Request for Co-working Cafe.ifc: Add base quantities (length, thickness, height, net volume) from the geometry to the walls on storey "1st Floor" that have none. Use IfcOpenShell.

First a look at what the model holds.

```python
import ifcopenshell
import ifcopenshell.util.element
import ifcopenshell.util.unit

model = ifcopenshell.open("Co-working Cafe.ifc")
print(model.schema)
for unit_type in ("LENGTHUNIT", "AREAUNIT", "VOLUMEUNIT"):
    print(unit_type, ifcopenshell.util.unit.calculate_unit_scale(model, unit_type))
storey = next(s for s in model.by_type("IfcBuildingStorey") if s.Name == "1st Floor")
walls = [e for e in ifcopenshell.util.element.get_decomposition(storey) if e.is_a("IfcWall")]
for e in sorted(walls, key=lambda e: e.id()):
    print(e.id(), e.is_a(), e.Name, list(ifcopenshell.util.element.get_psets(e, qtos_only=True)), sep=" | ")
```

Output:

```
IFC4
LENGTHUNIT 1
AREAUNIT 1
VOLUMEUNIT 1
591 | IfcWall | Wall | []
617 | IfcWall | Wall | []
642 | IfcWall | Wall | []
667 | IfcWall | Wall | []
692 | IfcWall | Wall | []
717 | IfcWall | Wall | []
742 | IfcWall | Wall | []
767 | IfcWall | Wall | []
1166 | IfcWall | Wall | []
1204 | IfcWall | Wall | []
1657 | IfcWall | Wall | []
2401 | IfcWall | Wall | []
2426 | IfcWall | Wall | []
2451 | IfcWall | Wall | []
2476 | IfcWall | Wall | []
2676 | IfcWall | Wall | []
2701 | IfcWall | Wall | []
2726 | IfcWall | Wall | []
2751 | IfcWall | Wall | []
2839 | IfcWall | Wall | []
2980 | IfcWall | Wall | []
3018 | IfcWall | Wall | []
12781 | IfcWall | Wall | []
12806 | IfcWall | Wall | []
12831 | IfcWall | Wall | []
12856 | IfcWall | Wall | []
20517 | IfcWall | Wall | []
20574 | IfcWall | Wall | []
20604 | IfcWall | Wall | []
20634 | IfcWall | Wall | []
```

```python
import ifcopenshell
import ifcopenshell.api.pset
import ifcopenshell.geom
import ifcopenshell.util.element
import ifcopenshell.util.shape
import ifcopenshell.util.unit

model = ifcopenshell.open("Co-working Cafe.ifc")
unit_scale = ifcopenshell.util.unit.calculate_unit_scale(model)
volume_scale = ifcopenshell.util.unit.calculate_unit_scale(model, "VOLUMEUNIT")
settings = ifcopenshell.geom.settings()

storey = next(s for s in model.by_type("IfcBuildingStorey") if s.Name == "1st Floor")
walls = [e for e in ifcopenshell.util.element.get_decomposition(storey) if e.is_a("IfcWall")]

for e in sorted(walls, key=lambda e: e.id()):
    if ifcopenshell.util.element.get_psets(e, qtos_only=True, should_inherit=False):
        continue
    # Geometry comes back in metres, in the element's own axes.
    shape = ifcopenshell.geom.create_shape(settings, e)
    values = {
        "Length": ifcopenshell.util.shape.get_x(shape.geometry) / unit_scale,
        "Width": ifcopenshell.util.shape.get_y(shape.geometry) / unit_scale,
        "Height": ifcopenshell.util.shape.get_z(shape.geometry) / unit_scale,
        "NetVolume": ifcopenshell.util.shape.get_volume(shape.geometry) / volume_scale,
    }
    qto = ifcopenshell.api.pset.add_qto(model, product=e, name="Qto_WallBaseQuantities")
    ifcopenshell.api.pset.edit_qto(model, qto=qto, properties=values)
    print(e.id(), {k: round(v, 3) for k, v in values.items()})

model.write("Co-working Cafe-out.ifc")
```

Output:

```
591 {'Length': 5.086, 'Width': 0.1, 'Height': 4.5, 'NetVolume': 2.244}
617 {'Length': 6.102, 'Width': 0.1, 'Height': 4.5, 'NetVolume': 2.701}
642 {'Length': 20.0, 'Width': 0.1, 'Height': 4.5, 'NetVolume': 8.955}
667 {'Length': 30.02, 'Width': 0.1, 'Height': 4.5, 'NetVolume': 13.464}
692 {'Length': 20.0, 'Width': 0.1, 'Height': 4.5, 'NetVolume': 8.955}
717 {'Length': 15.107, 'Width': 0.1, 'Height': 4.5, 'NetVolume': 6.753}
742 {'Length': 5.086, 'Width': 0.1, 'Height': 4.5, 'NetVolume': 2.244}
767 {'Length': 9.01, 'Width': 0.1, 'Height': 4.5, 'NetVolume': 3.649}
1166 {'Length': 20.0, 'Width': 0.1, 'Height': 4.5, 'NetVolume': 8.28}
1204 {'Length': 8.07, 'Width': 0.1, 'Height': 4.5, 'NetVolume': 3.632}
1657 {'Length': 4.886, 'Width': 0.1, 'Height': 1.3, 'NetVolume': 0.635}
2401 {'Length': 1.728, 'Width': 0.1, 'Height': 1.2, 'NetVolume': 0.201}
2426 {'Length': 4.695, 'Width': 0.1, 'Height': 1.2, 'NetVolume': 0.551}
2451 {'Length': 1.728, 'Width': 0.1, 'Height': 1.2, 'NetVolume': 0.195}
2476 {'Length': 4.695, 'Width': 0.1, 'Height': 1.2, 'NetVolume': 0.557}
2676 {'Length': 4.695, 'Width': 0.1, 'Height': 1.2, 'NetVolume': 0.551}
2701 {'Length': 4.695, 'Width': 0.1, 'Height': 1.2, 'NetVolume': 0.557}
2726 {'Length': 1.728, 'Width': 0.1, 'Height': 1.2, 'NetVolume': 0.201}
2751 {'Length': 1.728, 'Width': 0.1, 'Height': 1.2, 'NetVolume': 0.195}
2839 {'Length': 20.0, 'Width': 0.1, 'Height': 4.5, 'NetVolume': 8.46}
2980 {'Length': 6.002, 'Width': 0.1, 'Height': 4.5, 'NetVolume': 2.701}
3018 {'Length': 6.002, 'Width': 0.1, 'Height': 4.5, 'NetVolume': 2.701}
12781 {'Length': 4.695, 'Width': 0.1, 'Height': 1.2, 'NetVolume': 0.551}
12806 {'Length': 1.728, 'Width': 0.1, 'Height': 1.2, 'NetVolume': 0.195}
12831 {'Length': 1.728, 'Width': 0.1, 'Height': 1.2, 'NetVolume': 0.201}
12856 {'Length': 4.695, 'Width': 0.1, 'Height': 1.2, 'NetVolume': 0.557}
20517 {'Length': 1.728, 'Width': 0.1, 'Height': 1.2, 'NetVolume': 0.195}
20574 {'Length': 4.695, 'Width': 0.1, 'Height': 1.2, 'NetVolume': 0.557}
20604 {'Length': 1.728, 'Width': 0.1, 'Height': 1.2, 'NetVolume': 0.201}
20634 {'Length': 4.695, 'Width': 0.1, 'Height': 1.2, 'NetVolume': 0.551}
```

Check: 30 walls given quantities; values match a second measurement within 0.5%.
